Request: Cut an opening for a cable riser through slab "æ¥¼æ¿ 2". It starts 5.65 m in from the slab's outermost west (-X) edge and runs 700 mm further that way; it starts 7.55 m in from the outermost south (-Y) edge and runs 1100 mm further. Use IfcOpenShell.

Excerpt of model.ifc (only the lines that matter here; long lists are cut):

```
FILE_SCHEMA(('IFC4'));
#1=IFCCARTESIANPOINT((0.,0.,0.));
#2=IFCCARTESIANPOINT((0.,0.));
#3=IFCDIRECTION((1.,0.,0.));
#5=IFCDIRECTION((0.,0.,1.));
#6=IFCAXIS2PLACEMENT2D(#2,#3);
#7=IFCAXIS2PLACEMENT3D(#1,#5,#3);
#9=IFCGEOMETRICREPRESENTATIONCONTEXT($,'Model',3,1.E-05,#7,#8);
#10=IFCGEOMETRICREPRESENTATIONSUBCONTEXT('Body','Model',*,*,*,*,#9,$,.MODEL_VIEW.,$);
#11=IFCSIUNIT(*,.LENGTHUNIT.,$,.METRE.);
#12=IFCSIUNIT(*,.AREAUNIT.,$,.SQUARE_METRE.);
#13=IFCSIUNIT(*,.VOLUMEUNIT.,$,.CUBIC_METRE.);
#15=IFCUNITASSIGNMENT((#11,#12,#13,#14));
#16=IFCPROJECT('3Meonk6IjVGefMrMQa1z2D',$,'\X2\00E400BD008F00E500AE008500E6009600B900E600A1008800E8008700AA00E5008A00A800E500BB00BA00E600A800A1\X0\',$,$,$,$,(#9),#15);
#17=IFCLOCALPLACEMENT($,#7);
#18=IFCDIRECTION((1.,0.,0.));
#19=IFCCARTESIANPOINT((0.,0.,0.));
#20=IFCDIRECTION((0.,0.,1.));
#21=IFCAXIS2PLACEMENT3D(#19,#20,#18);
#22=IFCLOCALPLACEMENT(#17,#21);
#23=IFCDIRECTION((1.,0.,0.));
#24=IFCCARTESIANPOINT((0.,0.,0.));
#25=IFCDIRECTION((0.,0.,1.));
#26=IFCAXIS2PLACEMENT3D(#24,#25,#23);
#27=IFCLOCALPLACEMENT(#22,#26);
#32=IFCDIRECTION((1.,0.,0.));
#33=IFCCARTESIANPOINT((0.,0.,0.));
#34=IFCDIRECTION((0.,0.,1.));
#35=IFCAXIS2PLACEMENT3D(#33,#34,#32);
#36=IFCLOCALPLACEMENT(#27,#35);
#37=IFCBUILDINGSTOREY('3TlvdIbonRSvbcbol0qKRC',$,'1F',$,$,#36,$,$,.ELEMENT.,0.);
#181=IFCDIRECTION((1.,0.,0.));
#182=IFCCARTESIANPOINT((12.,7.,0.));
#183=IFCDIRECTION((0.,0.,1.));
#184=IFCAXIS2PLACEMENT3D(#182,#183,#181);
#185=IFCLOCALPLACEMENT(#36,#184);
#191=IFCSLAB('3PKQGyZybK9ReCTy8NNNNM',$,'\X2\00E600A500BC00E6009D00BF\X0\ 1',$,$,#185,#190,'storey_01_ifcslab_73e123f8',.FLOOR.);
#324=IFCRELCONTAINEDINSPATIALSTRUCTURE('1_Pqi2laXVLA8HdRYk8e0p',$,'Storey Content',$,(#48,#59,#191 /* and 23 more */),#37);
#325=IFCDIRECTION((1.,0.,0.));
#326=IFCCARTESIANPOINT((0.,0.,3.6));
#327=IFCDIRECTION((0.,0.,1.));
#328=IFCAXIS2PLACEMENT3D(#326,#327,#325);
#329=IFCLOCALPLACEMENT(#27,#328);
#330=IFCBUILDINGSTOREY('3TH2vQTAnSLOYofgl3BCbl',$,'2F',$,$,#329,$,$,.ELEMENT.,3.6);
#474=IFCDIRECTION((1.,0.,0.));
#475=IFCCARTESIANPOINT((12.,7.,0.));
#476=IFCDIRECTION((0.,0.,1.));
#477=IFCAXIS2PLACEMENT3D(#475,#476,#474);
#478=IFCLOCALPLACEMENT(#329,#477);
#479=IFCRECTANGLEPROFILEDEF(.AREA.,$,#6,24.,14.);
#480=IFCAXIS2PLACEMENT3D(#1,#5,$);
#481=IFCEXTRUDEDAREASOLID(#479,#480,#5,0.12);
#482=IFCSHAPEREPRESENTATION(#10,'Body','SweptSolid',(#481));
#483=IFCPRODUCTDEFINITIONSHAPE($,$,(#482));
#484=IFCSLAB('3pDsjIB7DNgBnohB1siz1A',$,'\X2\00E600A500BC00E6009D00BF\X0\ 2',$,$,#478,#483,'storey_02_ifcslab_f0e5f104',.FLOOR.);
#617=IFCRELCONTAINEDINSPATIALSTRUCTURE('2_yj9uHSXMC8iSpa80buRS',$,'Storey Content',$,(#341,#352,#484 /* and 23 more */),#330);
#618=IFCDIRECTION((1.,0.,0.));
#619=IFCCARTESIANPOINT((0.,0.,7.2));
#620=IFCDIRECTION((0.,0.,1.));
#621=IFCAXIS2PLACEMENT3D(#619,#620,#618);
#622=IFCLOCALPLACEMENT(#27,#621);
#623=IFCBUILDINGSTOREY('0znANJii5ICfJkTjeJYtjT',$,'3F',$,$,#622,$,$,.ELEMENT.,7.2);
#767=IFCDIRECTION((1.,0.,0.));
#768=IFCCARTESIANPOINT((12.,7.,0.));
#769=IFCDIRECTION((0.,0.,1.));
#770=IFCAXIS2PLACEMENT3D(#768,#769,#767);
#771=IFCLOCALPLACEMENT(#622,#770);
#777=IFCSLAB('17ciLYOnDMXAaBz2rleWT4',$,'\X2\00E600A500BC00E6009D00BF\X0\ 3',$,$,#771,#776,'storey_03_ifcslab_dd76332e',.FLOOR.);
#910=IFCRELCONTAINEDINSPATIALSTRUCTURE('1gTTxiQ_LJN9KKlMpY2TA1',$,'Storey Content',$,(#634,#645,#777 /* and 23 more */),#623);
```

```python
import numpy as np
import ifcopenshell
import ifcopenshell.api.feature
import ifcopenshell.api.geometry
import ifcopenshell.api.root
import ifcopenshell.geom
import ifcopenshell.util.placement
import ifcopenshell.util.representation
import ifcopenshell.util.shape
import ifcopenshell.util.unit

model = ifcopenshell.open("model.ifc")
unit_scale = ifcopenshell.util.unit.calculate_unit_scale(model)
settings = ifcopenshell.geom.settings()


def volume(element):
    """Net volume in cubic metres, openings subtracted."""
    shape = ifcopenshell.geom.create_shape(settings, element)
    return ifcopenshell.util.shape.get_volume(shape.geometry)


slab = model.by_guid("3pDsjIB7DNgBnohB1siz1A")
before = volume(slab)

# Extent in the slab's own axes, in metres. The edges named are its -X and -Y sides.
slab_shape = ifcopenshell.geom.create_shape(settings, slab)
vertices = ifcopenshell.util.shape.get_vertices(slab_shape.geometry)
x_min, y_min, bottom = vertices.min(axis=0)
top = vertices[:, 2].max()

opening = ifcopenshell.api.root.create_entity(model, ifc_class="IfcOpeningElement", name="Cable riser opening", predefined_type="OPENING")
context = ifcopenshell.util.representation.get_context(model, "Model", "Body", "MODEL_VIEW")
width, depth = 0.7, 1.1
outline = [(0.0, 0.0), (width, 0.0), (width, depth), (0.0, depth), (0.0, 0.0)]
# Overshoot both faces by 50 mm so the cut is clean.
shape = ifcopenshell.api.geometry.add_slab_representation(
    model, context=context, depth=top - bottom + 0.1, polyline=outline
)
ifcopenshell.api.geometry.assign_representation(model, product=opening, representation=shape)

matrix = ifcopenshell.util.placement.get_local_placement(slab.ObjectPlacement)
matrix[:, 3] = matrix @ np.append(np.array([x_min + 5.65, y_min + 7.55, bottom - 0.05]) / unit_scale, 1.0)
ifcopenshell.api.geometry.edit_object_placement(model, product=opening, matrix=matrix, is_si=False)
ifcopenshell.api.feature.add_feature(model, feature=opening, element=slab)

after = volume(slab)

print(f"slab volume {before:.3f} -> {after:.3f} m3")

model.write("model_v2.ifc")
```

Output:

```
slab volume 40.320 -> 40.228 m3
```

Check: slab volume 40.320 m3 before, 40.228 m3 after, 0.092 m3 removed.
